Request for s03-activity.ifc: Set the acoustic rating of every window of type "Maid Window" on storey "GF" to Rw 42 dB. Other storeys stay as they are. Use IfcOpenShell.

First a look at what the model holds.

```python
import ifcopenshell
import ifcopenshell.util.element

model = ifcopenshell.open("s03-activity.ifc")
print(model.schema)
storey = next(s for s in model.by_type("IfcBuildingStorey") if s.Name == "GF")
windows = [e for e in ifcopenshell.util.element.get_decomposition(storey) if e.is_a("IfcWindow")]
seen = {}
for e in windows:
    element_type = ifcopenshell.util.element.get_type(e)
    key = (element_type.Name if element_type != e and element_type else None, ifcopenshell.util.element.get_pset(e, "Pset_WindowCommon", "AcousticRating"))
    seen[key] = seen.get(key, 0) + 1
for (name, value), count in sorted(seen.items(), key=str):
    print(count, "x", name, "|", value)
```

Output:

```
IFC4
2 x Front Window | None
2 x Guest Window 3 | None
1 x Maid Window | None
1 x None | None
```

```python
import ifcopenshell
import ifcopenshell.api.pset
import ifcopenshell.util.element

model = ifcopenshell.open("s03-activity.ifc")

storey = next(s for s in model.by_type("IfcBuildingStorey") if s.Name == "GF")
windows = [e for e in ifcopenshell.util.element.get_decomposition(storey) if e.is_a("IfcWindow")]

count = 0
for e in windows:
    element_type = ifcopenshell.util.element.get_type(e)
    if element_type in (None, e) or element_type.Name != "Maid Window":
        continue
    # add_pset returns the element's existing set when there is one.
    pset = ifcopenshell.api.pset.add_pset(model, product=e, name="Pset_WindowCommon")
    ifcopenshell.api.pset.edit_pset(model, pset=pset, properties={"AcousticRating": "Rw 42 dB"})
    count += 1

print(count, "windows updated")

model.write("s03-activity_rev.ifc")
```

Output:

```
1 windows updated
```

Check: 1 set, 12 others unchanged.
